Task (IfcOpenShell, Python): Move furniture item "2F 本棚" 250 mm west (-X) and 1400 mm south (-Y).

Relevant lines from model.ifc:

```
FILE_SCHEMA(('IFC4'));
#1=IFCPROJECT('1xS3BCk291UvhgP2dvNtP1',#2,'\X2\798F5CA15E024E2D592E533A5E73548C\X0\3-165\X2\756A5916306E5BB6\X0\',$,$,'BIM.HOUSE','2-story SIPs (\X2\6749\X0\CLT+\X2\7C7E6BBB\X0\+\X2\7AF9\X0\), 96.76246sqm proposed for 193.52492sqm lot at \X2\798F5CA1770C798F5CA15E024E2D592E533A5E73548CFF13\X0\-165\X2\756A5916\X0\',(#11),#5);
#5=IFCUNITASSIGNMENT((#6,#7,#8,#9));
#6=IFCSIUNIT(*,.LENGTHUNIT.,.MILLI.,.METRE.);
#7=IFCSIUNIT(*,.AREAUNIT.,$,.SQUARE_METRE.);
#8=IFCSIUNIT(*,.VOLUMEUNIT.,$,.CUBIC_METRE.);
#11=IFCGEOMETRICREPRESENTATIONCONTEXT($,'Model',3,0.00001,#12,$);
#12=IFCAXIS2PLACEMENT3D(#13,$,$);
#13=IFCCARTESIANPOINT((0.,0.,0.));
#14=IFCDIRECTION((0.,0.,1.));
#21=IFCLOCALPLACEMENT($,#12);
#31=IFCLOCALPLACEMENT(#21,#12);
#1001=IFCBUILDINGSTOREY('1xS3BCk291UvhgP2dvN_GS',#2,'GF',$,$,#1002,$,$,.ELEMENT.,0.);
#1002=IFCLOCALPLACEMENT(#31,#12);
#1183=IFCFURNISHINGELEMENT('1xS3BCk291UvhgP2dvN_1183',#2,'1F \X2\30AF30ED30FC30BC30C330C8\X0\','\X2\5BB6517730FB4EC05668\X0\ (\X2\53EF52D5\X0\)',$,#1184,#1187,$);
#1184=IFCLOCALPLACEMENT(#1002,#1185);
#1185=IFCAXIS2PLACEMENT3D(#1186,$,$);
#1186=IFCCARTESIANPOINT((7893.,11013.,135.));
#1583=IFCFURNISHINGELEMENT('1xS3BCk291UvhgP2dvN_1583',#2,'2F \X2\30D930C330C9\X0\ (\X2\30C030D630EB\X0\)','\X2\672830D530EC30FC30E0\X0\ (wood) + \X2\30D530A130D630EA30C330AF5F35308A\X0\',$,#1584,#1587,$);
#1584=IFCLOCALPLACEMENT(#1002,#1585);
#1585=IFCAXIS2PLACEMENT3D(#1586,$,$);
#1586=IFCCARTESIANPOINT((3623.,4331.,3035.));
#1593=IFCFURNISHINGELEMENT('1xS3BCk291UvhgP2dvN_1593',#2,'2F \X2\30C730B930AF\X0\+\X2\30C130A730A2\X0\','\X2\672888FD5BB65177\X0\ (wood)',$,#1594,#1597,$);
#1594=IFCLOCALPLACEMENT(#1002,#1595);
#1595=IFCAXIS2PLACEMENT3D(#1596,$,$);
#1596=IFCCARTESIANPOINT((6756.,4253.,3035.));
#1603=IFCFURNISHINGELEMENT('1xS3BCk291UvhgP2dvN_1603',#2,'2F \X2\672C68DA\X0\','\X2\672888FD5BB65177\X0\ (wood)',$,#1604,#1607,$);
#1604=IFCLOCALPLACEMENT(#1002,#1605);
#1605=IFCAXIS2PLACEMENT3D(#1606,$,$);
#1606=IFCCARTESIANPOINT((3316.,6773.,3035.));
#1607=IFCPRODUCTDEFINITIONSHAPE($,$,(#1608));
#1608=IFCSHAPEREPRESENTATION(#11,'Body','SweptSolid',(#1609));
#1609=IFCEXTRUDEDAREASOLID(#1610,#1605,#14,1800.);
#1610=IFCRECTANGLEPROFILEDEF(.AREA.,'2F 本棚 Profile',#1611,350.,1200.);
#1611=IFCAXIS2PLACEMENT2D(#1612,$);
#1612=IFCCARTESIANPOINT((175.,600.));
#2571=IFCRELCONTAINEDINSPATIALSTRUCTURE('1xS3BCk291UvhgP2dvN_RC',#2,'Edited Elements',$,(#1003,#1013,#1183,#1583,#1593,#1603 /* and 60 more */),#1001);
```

```python
import ifcopenshell
import ifcopenshell.api.geometry
import ifcopenshell.util.placement
import ifcopenshell.util.unit

model = ifcopenshell.open("model.ifc")
unit_scale = ifcopenshell.util.unit.calculate_unit_scale(model)

item = model.by_guid("1xS3BCk291UvhgP2dvN_1603")
matrix = ifcopenshell.util.placement.get_local_placement(item.ObjectPlacement)
matrix[0, 3] -= 0.25 / unit_scale
matrix[1, 3] -= 1.4 / unit_scale
ifcopenshell.api.geometry.edit_object_placement(model, product=item, matrix=matrix, is_si=False)

print(ifcopenshell.util.placement.get_local_placement(item.ObjectPlacement).round(3) + 0.0)

model.write("model-out.ifc")
```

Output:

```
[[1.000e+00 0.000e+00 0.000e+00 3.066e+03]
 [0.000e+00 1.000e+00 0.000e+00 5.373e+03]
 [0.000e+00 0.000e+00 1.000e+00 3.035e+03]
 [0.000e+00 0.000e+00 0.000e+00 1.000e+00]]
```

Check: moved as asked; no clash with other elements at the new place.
